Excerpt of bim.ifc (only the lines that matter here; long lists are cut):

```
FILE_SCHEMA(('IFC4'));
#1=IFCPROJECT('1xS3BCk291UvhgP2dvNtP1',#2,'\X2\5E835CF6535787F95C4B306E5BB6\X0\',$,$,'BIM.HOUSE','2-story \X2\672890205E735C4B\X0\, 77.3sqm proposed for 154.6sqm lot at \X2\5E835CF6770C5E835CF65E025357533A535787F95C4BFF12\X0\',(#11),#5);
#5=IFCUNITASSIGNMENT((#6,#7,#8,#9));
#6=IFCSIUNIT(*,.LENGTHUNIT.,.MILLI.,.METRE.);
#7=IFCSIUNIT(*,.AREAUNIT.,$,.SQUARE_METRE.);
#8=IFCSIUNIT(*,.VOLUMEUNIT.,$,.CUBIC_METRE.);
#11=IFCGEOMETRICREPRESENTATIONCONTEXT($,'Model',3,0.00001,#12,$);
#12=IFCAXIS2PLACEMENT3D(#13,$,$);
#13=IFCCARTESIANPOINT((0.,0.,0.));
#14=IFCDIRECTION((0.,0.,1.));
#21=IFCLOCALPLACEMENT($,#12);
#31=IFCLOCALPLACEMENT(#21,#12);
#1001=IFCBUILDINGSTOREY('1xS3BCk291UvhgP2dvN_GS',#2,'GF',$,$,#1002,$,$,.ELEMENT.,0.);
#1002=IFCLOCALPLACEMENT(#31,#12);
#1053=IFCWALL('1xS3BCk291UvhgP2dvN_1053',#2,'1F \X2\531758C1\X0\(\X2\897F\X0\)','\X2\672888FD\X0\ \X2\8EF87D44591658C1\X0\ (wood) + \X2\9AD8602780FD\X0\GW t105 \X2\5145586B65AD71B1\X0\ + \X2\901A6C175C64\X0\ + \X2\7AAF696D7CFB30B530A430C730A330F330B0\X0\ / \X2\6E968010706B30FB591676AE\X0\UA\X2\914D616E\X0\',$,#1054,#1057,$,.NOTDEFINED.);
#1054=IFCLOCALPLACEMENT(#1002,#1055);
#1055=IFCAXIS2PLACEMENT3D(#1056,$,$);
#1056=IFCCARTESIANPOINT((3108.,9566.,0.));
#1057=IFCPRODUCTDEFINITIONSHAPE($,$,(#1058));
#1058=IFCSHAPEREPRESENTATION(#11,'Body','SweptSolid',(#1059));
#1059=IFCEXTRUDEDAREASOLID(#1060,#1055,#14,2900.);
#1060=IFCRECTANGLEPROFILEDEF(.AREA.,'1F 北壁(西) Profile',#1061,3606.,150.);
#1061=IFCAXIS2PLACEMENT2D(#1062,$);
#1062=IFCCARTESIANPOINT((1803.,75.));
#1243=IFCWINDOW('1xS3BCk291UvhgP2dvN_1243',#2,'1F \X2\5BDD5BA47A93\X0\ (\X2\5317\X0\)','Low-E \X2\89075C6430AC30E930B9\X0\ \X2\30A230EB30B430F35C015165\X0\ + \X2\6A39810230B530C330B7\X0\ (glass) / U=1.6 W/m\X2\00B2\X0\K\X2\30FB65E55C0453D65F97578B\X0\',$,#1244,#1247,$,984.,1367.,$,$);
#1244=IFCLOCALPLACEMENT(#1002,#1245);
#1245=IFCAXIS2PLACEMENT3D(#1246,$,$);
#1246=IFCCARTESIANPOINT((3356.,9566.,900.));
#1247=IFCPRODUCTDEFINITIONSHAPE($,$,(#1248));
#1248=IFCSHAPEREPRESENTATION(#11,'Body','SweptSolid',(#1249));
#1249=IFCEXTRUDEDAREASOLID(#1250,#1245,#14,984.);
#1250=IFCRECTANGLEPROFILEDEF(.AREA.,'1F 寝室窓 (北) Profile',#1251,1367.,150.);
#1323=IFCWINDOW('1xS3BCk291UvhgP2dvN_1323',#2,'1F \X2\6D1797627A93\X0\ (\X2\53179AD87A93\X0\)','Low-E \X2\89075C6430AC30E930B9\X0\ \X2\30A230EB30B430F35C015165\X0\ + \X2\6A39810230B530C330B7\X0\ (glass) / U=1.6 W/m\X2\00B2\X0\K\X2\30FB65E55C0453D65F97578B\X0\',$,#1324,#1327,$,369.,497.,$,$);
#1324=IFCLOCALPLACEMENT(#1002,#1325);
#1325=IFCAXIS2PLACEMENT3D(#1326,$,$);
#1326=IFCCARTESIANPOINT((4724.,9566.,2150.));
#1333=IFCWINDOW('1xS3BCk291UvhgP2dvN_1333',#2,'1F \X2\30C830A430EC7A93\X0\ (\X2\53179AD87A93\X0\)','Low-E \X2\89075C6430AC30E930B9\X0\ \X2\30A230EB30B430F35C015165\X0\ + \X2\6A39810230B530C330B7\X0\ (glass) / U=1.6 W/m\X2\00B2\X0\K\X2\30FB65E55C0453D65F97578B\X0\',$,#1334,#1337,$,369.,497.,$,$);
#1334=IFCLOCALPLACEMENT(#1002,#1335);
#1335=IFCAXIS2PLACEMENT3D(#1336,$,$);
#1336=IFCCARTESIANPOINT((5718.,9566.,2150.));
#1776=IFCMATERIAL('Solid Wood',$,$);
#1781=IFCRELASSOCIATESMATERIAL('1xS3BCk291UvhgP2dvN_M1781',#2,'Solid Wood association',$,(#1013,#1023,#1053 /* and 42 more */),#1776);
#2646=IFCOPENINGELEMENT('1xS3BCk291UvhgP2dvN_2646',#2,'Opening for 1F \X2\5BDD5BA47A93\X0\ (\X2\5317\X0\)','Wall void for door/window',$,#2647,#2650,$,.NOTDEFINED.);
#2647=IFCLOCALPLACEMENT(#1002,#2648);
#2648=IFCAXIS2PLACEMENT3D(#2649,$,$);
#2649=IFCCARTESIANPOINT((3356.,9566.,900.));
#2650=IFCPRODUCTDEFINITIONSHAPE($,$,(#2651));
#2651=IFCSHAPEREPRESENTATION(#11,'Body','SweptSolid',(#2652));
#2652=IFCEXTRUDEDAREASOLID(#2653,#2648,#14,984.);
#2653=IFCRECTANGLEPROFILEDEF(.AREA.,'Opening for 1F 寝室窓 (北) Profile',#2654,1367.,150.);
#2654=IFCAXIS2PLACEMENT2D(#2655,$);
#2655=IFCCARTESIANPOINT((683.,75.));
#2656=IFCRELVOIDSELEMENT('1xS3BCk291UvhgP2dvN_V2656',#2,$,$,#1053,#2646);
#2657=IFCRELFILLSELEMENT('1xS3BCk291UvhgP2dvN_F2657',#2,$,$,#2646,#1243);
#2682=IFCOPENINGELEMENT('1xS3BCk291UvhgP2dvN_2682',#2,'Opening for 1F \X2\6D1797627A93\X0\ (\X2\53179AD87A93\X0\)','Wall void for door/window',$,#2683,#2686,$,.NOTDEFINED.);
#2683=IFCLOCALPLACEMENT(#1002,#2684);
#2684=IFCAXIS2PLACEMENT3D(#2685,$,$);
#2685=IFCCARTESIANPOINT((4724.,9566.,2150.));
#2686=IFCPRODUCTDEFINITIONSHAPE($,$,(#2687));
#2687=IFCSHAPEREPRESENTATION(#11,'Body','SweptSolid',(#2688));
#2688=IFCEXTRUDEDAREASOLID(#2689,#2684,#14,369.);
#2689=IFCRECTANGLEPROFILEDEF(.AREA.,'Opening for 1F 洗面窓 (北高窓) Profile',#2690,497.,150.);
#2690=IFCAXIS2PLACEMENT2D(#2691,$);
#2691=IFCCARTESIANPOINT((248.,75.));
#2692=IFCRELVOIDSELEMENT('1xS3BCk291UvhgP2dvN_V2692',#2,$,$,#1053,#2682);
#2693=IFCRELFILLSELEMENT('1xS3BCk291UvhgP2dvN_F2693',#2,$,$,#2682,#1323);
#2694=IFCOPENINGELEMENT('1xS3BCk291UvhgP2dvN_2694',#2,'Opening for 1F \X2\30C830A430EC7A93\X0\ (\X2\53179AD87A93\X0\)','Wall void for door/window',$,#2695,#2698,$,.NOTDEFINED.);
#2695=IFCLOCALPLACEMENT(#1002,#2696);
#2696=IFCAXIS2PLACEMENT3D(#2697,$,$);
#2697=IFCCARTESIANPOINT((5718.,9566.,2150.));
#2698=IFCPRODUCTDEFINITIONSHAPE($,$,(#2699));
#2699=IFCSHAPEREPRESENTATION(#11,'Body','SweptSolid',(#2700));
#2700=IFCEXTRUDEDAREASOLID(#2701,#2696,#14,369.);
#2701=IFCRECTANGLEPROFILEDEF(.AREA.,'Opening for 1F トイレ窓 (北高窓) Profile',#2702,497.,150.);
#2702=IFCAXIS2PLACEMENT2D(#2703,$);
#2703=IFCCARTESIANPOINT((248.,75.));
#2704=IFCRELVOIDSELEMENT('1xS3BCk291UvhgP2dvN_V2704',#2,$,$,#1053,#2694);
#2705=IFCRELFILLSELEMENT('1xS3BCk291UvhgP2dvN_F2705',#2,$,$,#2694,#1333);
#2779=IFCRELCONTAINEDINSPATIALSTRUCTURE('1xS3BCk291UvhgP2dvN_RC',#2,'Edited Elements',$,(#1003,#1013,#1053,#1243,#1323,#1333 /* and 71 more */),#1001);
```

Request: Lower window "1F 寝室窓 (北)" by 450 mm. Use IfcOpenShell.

```python
import numpy as np
import ifcopenshell
import ifcopenshell.api.geometry
import ifcopenshell.util.placement
import ifcopenshell.util.unit

model = ifcopenshell.open("bim.ifc")
unit_scale = ifcopenshell.util.unit.calculate_unit_scale(model)

window = model.by_id(1243)
opening = window.FillsVoids[0].RelatingOpeningElement
dz = -450.0

shift = np.array([0.0, 0.0, dz])
# The window is not placed relative to its opening, so move both.
for product in (opening, window):
    matrix = ifcopenshell.util.placement.get_local_placement(product.ObjectPlacement)
    matrix[:3, 3] += shift
    ifcopenshell.api.geometry.edit_object_placement(model, product=product, matrix=matrix, is_si=False)

print(f"moved by {dz * unit_scale:+.3f} m")

model.write("bim_rev.ifc")
```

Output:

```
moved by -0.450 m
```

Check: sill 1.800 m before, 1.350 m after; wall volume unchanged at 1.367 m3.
